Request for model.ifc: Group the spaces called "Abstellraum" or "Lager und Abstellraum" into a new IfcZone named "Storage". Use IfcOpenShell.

First a look at what the model holds.

```python
import ifcopenshell

model = ifcopenshell.open("model.ifc")
print(model.schema)
seen = {}
for space in model.by_type("IfcSpace"):
    seen[space.LongName] = seen.get(space.LongName, 0) + 1
for name, count in sorted(seen.items(), key=str):
    print(count, "x", name)
print("zones:", [z.Name for z in model.by_type("IfcZone")][:20])
```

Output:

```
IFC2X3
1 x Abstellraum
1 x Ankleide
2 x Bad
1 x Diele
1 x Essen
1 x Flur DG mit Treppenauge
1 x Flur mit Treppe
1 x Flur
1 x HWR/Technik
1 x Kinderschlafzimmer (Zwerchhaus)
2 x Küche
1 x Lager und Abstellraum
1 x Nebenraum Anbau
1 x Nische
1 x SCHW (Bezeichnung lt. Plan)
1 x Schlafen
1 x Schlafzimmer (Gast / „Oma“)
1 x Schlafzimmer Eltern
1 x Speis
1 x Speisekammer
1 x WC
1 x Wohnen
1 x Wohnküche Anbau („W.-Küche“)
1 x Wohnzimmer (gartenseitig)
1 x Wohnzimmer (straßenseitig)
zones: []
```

```python
import ifcopenshell
import ifcopenshell.api.group
import ifcopenshell.api.root

model = ifcopenshell.open("model.ifc")

names = {"Abstellraum", "Lager und Abstellraum"}
spaces = [s for s in model.by_type("IfcSpace") if s.LongName in names]

zone = ifcopenshell.api.root.create_entity(model, ifc_class="IfcZone", name="Storage")
ifcopenshell.api.group.assign_group(model, products=spaces, group=zone)
print(len(spaces), "spaces in", zone.Name)

model.write("model_rev.ifc")
```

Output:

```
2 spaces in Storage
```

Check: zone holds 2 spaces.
